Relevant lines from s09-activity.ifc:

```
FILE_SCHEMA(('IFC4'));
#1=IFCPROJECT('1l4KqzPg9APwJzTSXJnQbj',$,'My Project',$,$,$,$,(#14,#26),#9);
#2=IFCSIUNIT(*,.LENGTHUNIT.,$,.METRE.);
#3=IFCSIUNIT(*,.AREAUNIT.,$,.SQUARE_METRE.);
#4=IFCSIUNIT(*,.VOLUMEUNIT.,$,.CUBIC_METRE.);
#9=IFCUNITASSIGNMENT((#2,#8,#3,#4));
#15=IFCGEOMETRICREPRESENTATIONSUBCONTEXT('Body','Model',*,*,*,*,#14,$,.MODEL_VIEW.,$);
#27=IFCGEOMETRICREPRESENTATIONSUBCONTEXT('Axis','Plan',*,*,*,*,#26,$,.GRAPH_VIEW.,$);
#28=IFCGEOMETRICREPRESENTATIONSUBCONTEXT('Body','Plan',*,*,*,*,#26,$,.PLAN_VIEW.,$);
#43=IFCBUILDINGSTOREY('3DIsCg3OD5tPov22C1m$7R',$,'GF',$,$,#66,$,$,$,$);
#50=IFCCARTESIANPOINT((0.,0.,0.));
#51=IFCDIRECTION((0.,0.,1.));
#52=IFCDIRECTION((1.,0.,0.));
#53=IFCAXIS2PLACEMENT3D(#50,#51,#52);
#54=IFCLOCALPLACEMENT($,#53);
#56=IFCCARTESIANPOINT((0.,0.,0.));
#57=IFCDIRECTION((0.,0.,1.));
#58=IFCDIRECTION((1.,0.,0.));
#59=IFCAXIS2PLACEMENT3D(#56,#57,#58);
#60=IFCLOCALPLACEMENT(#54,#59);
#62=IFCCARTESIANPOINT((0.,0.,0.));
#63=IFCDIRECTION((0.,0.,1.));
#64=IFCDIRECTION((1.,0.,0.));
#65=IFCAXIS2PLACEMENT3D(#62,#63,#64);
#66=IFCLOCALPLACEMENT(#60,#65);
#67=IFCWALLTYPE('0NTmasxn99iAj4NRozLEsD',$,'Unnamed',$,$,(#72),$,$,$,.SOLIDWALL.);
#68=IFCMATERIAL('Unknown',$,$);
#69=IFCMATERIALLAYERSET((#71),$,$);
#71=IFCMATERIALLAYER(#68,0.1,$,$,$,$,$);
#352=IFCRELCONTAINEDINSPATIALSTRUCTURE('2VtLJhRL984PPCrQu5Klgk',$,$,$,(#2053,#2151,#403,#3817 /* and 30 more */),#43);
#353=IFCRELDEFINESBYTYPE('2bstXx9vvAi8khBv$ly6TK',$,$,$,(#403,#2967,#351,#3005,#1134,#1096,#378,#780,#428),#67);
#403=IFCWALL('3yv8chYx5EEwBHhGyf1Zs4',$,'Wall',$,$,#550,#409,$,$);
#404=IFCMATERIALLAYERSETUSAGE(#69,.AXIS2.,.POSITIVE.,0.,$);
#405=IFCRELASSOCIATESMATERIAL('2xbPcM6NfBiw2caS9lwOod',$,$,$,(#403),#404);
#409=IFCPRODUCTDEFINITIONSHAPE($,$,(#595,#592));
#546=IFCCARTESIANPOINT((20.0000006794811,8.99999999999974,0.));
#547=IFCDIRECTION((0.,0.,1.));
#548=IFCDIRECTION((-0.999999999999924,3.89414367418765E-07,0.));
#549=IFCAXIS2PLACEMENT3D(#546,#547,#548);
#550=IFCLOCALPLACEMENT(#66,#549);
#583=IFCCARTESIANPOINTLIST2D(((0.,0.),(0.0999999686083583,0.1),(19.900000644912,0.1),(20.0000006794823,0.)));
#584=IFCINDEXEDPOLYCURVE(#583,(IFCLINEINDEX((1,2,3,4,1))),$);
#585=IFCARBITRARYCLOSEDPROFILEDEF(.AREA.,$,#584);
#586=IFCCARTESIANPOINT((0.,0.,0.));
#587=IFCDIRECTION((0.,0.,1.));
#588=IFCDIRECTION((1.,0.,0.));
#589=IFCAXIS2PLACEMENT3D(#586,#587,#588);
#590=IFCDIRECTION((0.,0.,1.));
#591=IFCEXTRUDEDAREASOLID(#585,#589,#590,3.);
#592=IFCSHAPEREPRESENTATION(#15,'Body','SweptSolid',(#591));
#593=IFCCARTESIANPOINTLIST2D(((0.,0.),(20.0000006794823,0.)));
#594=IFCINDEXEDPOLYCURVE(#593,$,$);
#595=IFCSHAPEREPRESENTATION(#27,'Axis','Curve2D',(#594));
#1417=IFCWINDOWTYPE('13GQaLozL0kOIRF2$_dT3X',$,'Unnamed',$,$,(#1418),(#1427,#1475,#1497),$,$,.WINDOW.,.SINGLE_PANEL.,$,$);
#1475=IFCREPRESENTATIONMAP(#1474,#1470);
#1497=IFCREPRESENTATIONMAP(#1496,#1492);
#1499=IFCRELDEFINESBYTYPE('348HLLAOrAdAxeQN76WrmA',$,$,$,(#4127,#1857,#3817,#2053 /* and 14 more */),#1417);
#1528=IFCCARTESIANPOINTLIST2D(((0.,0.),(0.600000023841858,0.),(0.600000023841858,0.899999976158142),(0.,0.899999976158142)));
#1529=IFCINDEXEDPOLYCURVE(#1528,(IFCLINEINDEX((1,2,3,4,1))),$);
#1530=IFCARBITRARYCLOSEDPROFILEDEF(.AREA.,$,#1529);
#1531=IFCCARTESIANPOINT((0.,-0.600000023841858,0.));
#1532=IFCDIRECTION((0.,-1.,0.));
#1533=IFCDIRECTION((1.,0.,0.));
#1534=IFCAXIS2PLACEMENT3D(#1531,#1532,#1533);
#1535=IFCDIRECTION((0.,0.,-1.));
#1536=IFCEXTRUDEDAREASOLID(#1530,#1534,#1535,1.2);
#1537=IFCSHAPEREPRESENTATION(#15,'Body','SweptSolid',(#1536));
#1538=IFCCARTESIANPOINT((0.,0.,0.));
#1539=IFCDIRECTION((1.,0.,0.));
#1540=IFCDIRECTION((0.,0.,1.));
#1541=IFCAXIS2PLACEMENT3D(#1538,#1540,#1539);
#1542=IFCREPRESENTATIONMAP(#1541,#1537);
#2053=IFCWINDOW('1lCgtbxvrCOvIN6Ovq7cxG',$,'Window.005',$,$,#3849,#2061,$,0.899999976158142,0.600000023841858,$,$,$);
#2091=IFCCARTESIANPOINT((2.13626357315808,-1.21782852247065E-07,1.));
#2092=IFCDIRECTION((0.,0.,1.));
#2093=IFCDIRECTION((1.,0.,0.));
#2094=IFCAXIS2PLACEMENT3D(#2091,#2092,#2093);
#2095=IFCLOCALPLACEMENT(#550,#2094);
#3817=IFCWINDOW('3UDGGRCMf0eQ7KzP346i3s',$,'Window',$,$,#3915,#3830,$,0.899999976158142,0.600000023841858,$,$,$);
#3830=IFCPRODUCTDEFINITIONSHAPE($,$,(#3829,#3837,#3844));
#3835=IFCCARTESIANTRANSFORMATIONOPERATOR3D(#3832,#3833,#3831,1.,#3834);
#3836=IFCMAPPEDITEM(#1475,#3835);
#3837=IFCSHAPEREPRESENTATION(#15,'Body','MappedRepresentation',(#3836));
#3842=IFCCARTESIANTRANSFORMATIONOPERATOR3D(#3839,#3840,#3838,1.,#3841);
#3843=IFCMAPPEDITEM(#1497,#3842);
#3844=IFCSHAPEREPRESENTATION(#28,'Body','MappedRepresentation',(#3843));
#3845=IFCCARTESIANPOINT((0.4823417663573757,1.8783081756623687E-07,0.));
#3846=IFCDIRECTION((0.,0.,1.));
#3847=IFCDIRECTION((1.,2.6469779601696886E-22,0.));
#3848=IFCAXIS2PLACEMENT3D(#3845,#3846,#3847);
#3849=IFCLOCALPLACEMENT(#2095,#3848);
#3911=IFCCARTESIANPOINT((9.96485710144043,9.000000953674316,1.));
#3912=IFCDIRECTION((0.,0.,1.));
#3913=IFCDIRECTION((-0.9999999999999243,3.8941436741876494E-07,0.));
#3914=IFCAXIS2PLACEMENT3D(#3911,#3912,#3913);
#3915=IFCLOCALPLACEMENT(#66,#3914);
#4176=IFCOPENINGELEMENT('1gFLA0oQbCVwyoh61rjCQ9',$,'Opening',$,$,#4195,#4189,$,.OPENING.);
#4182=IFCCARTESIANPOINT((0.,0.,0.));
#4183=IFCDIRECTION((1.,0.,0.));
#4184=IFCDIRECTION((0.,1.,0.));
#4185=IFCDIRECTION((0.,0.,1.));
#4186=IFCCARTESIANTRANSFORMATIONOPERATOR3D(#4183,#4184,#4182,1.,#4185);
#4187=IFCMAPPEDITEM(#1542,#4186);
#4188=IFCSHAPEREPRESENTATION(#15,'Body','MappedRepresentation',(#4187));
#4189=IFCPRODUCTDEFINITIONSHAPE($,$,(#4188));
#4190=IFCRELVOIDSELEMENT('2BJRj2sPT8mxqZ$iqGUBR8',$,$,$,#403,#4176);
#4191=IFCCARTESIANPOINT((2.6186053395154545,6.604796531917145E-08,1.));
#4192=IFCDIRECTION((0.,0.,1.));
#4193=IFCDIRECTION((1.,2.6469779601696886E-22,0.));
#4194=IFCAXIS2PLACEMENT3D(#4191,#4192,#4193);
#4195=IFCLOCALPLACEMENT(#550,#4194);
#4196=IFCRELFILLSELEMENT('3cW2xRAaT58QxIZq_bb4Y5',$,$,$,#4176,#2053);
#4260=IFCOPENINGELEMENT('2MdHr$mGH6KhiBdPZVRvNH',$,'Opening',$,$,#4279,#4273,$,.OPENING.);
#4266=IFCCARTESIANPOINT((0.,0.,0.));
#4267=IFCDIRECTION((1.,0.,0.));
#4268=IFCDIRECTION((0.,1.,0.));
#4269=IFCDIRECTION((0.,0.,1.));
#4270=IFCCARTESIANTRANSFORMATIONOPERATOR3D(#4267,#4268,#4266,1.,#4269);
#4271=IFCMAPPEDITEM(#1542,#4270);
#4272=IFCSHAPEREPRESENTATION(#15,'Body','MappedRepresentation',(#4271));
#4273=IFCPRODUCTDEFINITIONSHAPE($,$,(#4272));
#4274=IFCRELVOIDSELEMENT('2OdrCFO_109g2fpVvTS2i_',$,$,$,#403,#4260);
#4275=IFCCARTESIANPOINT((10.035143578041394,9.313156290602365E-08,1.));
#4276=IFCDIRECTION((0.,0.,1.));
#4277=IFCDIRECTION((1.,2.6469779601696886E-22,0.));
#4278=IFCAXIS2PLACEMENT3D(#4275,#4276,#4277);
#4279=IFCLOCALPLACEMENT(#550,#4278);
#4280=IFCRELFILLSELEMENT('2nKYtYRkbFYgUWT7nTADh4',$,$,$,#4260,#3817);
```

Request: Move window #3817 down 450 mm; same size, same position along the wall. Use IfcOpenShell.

```python
import numpy as np
import ifcopenshell
import ifcopenshell.api.geometry
import ifcopenshell.util.placement
import ifcopenshell.util.unit

model = ifcopenshell.open("s09-activity.ifc")
unit_scale = ifcopenshell.util.unit.calculate_unit_scale(model)

window = model.by_id(3817)
opening = window.FillsVoids[0].RelatingOpeningElement
dz = -0.45 / unit_scale

shift = np.array([0.0, 0.0, dz])
# The window is not placed relative to its opening, so move both.
for product in (opening, window):
    matrix = ifcopenshell.util.placement.get_local_placement(product.ObjectPlacement)
    matrix[:3, 3] += shift
    ifcopenshell.api.geometry.edit_object_placement(model, product=product, matrix=matrix, is_si=False)

print(f"moved by {dz * unit_scale:+.3f} m")

model.write("s09-activity_rev.ifc")
```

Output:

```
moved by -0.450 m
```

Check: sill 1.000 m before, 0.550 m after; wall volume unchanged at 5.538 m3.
